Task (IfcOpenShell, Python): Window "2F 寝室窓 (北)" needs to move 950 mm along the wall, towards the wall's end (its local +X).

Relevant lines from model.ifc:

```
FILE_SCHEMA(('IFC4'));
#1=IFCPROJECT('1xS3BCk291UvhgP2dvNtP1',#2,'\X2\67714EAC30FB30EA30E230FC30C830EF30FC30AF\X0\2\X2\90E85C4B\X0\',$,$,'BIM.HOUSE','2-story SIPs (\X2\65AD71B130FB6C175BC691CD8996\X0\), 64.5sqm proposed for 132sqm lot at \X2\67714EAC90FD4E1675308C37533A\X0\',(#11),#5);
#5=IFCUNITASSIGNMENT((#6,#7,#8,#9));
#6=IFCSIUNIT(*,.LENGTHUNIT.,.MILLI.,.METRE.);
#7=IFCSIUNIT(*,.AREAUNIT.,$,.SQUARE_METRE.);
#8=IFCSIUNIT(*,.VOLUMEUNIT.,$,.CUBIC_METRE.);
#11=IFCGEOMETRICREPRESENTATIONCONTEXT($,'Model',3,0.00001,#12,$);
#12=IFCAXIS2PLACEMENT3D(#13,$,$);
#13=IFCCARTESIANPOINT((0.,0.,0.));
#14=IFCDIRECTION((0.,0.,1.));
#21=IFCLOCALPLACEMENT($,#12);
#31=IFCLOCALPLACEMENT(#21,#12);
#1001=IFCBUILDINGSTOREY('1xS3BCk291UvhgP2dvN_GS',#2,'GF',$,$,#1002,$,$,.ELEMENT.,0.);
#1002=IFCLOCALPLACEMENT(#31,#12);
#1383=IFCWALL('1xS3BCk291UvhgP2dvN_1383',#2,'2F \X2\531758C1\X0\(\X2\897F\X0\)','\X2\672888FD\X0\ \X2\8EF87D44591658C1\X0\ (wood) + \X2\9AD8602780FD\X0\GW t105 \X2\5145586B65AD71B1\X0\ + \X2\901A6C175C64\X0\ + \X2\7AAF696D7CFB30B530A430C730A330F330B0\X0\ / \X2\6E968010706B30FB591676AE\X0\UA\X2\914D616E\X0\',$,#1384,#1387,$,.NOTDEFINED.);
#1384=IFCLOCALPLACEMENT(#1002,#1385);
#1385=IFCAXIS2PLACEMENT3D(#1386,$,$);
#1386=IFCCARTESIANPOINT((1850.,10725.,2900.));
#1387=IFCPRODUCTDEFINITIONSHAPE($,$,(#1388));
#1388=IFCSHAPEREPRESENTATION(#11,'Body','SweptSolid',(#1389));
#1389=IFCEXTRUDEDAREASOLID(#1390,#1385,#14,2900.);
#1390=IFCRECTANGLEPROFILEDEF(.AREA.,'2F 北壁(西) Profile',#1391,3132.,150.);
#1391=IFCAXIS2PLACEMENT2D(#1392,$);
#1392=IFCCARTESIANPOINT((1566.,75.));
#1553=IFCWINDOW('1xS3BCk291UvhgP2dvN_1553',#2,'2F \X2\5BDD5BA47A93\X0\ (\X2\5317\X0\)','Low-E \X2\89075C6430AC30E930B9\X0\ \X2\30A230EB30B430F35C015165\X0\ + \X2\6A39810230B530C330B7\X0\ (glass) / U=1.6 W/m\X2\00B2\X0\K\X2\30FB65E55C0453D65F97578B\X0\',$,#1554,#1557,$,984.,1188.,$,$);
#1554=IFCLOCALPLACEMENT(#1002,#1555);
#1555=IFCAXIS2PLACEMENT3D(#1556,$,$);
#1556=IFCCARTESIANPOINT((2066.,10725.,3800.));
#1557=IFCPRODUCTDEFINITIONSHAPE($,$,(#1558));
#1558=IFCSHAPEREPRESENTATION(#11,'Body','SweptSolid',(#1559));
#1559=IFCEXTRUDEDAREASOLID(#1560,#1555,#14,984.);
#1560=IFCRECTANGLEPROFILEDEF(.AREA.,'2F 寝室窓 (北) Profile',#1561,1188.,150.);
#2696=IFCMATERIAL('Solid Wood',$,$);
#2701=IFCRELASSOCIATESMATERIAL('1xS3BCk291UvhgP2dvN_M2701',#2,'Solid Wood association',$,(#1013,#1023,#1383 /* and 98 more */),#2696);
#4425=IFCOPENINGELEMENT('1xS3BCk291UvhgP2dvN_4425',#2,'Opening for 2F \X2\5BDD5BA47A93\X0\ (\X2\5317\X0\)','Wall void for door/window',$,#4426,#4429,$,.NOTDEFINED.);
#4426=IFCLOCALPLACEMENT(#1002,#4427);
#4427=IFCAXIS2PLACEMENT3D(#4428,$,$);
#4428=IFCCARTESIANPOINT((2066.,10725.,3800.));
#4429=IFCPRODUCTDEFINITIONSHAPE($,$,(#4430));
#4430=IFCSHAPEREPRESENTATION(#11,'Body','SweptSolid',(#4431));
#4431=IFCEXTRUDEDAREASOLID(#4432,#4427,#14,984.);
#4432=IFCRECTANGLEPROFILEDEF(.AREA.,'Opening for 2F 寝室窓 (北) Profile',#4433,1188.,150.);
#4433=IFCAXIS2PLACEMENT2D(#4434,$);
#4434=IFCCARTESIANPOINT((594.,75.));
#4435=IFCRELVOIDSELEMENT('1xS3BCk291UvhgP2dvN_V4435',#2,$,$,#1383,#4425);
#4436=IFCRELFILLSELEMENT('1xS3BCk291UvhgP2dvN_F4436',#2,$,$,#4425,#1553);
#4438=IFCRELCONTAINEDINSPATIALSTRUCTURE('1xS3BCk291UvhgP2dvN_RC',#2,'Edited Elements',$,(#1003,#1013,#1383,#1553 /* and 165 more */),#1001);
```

```python
import ifcopenshell
import ifcopenshell.api.geometry
import ifcopenshell.util.placement

model = ifcopenshell.open("model.ifc")

window = model.by_guid("1xS3BCk291UvhgP2dvN_1553")
opening = window.FillsVoids[0].RelatingOpeningElement
wall = opening.VoidsElements[0].RelatingBuildingElement

wall_matrix = ifcopenshell.util.placement.get_local_placement(wall.ObjectPlacement)
shift = wall_matrix[:3, 0] * 950.0
before = ifcopenshell.util.placement.get_local_placement(window.ObjectPlacement)[:3, 3].copy()

# The window is not placed relative to its opening, so move both.
for product in (opening, window):
    matrix = ifcopenshell.util.placement.get_local_placement(product.ObjectPlacement)
    matrix[:3, 3] += shift
    ifcopenshell.api.geometry.edit_object_placement(model, product=product, matrix=matrix, is_si=False)

after = ifcopenshell.util.placement.get_local_placement(window.ObjectPlacement)[:3, 3]
print("window moved by", (after - before).round(3) + 0.0)

model.write("model_edited.ifc")
```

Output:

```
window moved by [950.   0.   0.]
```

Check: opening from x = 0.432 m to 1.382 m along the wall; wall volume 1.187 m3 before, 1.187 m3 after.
